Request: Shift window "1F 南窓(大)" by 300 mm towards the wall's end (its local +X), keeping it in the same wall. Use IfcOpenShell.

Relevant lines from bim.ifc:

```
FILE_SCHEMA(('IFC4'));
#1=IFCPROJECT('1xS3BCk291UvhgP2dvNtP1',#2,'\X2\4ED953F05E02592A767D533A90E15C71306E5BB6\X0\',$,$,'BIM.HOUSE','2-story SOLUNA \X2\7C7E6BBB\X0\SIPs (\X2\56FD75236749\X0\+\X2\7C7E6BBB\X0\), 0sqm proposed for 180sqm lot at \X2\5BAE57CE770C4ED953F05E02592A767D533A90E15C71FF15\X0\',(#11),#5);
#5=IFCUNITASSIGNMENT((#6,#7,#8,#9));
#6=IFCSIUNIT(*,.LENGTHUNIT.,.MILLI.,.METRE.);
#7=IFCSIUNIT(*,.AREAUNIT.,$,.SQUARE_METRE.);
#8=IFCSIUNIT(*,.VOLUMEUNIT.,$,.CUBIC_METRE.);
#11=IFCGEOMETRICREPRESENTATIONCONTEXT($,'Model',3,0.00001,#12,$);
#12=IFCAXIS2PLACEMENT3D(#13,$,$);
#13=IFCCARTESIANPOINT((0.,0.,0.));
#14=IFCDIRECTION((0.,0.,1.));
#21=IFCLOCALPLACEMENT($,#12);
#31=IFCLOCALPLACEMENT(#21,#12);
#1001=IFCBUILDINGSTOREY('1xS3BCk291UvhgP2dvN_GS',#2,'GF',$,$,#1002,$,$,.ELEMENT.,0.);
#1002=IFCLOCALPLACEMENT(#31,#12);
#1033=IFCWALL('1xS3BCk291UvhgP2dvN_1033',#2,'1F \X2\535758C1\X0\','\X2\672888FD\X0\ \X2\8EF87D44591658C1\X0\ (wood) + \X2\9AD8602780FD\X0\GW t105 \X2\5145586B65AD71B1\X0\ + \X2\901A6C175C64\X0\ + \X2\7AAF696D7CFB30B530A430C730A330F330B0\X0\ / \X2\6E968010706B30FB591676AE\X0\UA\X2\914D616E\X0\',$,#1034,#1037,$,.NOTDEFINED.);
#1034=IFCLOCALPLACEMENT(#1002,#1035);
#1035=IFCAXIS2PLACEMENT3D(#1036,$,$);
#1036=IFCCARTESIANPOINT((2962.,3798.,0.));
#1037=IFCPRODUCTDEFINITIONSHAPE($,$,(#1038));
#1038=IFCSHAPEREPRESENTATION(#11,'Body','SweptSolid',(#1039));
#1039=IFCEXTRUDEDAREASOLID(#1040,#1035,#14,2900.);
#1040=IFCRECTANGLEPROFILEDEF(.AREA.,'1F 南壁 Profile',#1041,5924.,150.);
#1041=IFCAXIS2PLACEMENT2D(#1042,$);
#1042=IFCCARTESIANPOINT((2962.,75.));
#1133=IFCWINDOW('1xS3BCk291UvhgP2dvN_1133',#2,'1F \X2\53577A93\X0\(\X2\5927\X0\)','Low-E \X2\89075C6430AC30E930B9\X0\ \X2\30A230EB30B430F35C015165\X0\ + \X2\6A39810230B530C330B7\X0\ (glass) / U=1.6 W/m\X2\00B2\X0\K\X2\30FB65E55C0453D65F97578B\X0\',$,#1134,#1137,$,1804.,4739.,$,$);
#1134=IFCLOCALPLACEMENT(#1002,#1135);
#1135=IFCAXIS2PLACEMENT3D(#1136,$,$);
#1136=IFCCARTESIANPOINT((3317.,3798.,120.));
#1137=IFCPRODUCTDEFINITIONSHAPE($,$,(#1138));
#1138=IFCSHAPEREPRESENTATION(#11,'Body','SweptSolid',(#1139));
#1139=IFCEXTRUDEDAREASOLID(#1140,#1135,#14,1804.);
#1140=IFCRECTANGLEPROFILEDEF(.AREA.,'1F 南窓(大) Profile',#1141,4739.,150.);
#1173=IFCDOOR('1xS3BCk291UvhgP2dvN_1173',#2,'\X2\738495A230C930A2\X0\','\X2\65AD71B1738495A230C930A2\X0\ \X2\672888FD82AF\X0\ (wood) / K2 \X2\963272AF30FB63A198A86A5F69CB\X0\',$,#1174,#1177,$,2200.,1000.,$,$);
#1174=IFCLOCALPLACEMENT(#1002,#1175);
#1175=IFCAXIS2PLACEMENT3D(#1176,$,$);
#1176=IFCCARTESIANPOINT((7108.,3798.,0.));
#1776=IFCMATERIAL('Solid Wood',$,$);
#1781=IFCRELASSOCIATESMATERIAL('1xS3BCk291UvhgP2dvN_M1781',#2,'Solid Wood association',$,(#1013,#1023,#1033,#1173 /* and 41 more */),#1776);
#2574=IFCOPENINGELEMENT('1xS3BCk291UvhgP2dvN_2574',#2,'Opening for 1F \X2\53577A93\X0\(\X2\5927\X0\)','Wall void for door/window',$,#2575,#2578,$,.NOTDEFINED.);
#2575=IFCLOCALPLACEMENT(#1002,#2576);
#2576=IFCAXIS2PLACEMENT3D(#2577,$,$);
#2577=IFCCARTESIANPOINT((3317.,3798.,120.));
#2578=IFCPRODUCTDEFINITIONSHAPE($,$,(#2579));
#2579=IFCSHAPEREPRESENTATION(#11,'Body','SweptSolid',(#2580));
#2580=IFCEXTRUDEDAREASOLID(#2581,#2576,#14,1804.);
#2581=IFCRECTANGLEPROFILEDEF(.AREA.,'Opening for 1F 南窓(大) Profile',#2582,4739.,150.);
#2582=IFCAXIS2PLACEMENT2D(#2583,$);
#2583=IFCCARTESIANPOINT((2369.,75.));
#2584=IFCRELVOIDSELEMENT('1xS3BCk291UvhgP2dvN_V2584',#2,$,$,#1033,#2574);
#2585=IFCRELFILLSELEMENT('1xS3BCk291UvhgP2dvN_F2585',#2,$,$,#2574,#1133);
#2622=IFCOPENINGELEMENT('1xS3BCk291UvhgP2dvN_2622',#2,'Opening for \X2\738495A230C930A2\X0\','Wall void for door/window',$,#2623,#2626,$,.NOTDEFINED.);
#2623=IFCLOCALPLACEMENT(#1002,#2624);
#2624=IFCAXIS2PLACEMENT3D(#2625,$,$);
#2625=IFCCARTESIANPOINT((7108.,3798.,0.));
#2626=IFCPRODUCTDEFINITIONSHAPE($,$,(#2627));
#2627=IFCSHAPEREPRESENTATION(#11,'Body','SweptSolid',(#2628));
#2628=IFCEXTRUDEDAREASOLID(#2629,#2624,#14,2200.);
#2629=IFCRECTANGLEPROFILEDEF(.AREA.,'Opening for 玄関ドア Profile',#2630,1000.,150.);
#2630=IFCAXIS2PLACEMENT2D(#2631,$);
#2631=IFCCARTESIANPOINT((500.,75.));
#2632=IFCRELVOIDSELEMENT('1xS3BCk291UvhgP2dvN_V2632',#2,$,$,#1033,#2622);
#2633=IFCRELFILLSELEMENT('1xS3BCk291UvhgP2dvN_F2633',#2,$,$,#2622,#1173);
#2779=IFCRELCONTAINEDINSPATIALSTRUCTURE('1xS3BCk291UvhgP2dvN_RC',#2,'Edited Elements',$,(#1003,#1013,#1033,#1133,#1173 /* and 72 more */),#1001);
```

```python
import ifcopenshell
import ifcopenshell.api.geometry
import ifcopenshell.util.placement
import ifcopenshell.util.unit

model = ifcopenshell.open("bim.ifc")
unit_scale = ifcopenshell.util.unit.calculate_unit_scale(model)

window = model.by_guid("1xS3BCk291UvhgP2dvN_1133")
opening = window.FillsVoids[0].RelatingOpeningElement
wall = opening.VoidsElements[0].RelatingBuildingElement

wall_matrix = ifcopenshell.util.placement.get_local_placement(wall.ObjectPlacement)
shift = wall_matrix[:3, 0] * 0.3 / unit_scale
before = ifcopenshell.util.placement.get_local_placement(window.ObjectPlacement)[:3, 3].copy()

# The window is not placed relative to its opening, so move both.
for product in (opening, window):
    matrix = ifcopenshell.util.placement.get_local_placement(product.ObjectPlacement)
    matrix[:3, 3] += shift
    ifcopenshell.api.geometry.edit_object_placement(model, product=product, matrix=matrix, is_si=False)

after = ifcopenshell.util.placement.get_local_placement(window.ObjectPlacement)[:3, 3]
print("window moved by", (after - before).round(3) + 0.0)

model.write("bim-out.ifc")
```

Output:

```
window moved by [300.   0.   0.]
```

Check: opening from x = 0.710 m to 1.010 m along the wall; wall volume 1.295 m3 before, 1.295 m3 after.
